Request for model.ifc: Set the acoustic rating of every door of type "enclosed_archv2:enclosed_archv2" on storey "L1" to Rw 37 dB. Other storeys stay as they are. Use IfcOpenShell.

First a look at what the model holds.

```python
import ifcopenshell
import ifcopenshell.util.element

model = ifcopenshell.open("model.ifc")
print(model.schema)
storey = next(s for s in model.by_type("IfcBuildingStorey") if s.Name == "L1")
doors = [e for e in ifcopenshell.util.element.get_decomposition(storey) if e.is_a("IfcDoor")]
seen = {}
for e in doors:
    element_type = ifcopenshell.util.element.get_type(e)
    key = (element_type.Name if element_type != e and element_type else None, ifcopenshell.util.element.get_pset(e, "Pset_DoorCommon", "AcousticRating"))
    seen[key] = seen.get(key, 0) + 1
for (name, value), count in sorted(seen.items(), key=str):
    print(count, "x", name, "|", value)
```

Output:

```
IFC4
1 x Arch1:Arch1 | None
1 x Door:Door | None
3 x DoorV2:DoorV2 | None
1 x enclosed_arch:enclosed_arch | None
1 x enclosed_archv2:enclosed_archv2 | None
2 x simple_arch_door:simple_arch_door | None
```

```python
import ifcopenshell
import ifcopenshell.api.pset
import ifcopenshell.util.element

model = ifcopenshell.open("model.ifc")

storey = next(s for s in model.by_type("IfcBuildingStorey") if s.Name == "L1")
doors = [e for e in ifcopenshell.util.element.get_decomposition(storey) if e.is_a("IfcDoor")]

count = 0
for e in doors:
    element_type = ifcopenshell.util.element.get_type(e)
    if element_type in (None, e) or element_type.Name != "enclosed_archv2:enclosed_archv2":
        continue
    # add_pset returns the element's existing set when there is one.
    pset = ifcopenshell.api.pset.add_pset(model, product=e, name="Pset_DoorCommon")
    ifcopenshell.api.pset.edit_pset(model, pset=pset, properties={"AcousticRating": "Rw 37 dB"})
    count += 1

print(count, "doors updated")

model.write("model_updated.ifc")
```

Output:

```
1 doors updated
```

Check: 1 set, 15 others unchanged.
